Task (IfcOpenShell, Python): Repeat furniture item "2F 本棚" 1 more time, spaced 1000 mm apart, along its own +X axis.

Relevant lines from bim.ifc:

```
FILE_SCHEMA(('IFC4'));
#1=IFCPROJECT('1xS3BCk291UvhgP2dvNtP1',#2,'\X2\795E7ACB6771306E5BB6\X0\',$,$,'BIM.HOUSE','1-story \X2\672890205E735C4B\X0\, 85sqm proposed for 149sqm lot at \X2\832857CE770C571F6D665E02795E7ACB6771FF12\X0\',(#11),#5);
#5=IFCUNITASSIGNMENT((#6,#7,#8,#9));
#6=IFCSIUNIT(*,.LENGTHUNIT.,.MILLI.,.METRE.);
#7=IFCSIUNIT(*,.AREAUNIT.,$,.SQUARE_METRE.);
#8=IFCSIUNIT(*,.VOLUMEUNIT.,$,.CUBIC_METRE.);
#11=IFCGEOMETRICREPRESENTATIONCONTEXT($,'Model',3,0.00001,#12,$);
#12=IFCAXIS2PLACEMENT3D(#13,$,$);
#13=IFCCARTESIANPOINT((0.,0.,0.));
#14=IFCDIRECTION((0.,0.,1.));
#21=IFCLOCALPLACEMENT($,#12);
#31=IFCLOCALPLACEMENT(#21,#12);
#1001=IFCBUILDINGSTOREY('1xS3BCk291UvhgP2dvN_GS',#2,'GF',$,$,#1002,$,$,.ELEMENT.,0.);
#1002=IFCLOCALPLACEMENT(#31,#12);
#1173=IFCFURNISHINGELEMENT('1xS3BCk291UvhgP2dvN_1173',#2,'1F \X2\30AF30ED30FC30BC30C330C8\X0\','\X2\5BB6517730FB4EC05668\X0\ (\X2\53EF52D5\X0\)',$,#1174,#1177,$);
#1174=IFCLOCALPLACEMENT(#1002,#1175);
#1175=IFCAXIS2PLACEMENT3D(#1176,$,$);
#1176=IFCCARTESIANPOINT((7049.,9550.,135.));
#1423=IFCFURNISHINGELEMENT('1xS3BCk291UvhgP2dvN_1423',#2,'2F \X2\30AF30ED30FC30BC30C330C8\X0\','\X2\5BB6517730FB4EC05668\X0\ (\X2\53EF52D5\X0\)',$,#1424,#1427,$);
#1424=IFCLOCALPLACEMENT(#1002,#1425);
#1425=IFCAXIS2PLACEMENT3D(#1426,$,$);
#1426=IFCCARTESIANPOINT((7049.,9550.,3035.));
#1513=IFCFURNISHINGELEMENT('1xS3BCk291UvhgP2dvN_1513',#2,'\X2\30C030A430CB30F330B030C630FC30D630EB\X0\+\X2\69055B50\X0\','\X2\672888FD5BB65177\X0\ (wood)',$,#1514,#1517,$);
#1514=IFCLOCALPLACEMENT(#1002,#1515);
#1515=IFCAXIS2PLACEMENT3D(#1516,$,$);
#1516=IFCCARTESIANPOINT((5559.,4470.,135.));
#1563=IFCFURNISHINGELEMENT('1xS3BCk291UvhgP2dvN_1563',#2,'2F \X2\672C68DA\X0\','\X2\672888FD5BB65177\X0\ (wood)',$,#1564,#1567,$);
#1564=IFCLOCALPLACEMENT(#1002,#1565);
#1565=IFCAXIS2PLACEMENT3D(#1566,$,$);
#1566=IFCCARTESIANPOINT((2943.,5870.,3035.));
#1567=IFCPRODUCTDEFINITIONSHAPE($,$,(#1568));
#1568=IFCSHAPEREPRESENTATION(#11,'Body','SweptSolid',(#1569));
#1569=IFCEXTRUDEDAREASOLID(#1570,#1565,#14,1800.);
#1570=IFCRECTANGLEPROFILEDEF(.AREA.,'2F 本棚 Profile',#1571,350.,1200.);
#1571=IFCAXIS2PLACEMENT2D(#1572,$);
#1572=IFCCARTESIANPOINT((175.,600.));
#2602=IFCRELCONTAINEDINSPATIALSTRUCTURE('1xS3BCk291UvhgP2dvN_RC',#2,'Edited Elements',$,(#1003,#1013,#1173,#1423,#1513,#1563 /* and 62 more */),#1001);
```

```python
import ifcopenshell
import ifcopenshell.api.geometry
import ifcopenshell.api.root
import ifcopenshell.util.element
import ifcopenshell.util.placement
import ifcopenshell.util.unit

model = ifcopenshell.open("bim.ifc")
unit_scale = ifcopenshell.util.unit.calculate_unit_scale(model)


def reuse_history(source, copy):
    """copy_class also copies each property set's owner history, people and application; keep the originals."""
    for rel in copy.IsDefinedBy:
        if rel.is_a("IfcRelDefinesByProperties") and (history := rel.RelatingPropertyDefinition.OwnerHistory):
            rel.RelatingPropertyDefinition.OwnerHistory = source.OwnerHistory
            ifcopenshell.util.element.remove_deep2(model, history)


source = model.by_guid("1xS3BCk291UvhgP2dvN_1563")
base = ifcopenshell.util.placement.get_local_placement(source.ObjectPlacement)
step = base[:3, 0] * 1 / unit_scale

for i in range(1, 2):
    copy = ifcopenshell.api.root.copy_class(model, product=source)
    copy.Representation = ifcopenshell.util.element.copy_deep(
        model, source.Representation, exclude=["IfcGeometricRepresentationContext", "IfcRepresentationMap"]
    )
    reuse_history(source, copy)
    matrix = base.copy()
    matrix[:3, 3] += i * step
    print("added at", matrix[:3, 3].round(3) + 0.0)
    ifcopenshell.api.geometry.edit_object_placement(model, product=copy, matrix=matrix, is_si=False)

model.write("bim_edited.ifc")
```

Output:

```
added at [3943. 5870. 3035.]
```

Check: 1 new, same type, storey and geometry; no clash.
